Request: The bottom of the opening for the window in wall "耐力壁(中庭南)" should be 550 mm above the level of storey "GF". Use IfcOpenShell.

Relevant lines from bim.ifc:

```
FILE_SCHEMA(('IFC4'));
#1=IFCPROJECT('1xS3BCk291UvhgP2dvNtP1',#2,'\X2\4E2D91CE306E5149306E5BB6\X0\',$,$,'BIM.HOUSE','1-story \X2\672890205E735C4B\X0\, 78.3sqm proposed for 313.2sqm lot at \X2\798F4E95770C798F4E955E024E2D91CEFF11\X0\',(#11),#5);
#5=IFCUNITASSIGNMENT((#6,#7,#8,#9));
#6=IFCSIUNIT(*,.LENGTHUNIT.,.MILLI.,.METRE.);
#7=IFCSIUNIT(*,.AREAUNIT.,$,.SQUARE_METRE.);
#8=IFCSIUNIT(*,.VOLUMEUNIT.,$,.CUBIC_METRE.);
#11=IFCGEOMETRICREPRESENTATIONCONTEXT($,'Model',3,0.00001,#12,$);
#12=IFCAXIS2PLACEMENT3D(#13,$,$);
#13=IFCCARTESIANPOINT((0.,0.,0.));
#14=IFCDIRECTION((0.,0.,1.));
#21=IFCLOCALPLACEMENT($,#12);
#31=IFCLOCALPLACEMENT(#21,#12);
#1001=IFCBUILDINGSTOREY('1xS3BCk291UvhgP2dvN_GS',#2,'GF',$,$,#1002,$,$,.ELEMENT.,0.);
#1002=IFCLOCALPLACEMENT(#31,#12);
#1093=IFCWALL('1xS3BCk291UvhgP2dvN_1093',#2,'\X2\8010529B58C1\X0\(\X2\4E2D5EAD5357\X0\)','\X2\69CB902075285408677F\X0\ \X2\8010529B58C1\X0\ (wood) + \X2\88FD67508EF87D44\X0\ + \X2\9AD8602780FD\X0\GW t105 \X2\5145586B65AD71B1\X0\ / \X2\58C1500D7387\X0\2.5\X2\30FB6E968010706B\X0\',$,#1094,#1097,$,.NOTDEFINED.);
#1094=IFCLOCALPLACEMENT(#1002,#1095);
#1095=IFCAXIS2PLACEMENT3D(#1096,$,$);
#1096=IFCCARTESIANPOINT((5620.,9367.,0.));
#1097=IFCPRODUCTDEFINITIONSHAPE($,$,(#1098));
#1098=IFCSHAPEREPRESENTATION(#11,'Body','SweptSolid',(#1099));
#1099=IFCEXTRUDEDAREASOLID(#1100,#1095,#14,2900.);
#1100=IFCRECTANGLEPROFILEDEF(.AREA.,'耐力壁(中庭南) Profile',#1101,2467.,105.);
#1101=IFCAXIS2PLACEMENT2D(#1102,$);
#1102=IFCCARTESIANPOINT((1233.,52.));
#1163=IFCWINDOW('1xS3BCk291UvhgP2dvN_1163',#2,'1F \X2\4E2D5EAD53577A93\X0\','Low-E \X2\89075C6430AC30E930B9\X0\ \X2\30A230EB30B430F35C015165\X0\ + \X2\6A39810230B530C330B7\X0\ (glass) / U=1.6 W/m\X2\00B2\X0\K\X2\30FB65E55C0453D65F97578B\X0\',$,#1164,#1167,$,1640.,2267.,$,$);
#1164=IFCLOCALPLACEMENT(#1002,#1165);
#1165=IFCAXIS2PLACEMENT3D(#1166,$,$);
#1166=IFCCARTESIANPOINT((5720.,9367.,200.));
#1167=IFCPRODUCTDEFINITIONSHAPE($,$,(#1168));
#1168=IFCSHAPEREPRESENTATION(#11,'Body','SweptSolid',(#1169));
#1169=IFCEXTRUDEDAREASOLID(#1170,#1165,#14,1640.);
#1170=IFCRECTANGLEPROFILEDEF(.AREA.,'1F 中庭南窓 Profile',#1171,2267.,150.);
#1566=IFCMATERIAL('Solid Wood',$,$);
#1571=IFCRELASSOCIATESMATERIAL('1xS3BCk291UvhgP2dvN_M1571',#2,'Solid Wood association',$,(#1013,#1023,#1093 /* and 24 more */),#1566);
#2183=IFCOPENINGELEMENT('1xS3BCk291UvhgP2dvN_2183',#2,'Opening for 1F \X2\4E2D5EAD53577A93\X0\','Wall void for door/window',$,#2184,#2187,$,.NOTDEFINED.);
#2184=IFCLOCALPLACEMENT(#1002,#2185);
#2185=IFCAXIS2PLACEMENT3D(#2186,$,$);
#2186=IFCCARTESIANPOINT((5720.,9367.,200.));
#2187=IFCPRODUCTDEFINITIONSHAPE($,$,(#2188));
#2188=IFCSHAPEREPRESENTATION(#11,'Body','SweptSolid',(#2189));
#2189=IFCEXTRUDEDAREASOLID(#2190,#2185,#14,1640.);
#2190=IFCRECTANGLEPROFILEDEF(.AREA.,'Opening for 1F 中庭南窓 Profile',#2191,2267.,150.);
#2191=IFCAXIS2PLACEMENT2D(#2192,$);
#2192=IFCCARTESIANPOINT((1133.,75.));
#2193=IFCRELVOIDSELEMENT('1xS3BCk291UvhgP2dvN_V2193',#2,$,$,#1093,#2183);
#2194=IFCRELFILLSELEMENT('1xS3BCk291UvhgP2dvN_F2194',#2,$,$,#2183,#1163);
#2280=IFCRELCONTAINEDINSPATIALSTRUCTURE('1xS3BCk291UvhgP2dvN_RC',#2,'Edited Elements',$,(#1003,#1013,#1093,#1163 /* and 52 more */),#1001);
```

```python
import numpy as np
import ifcopenshell
import ifcopenshell.api.geometry
import ifcopenshell.geom
import ifcopenshell.util.element
import ifcopenshell.util.placement
import ifcopenshell.util.shape
import ifcopenshell.util.unit

model = ifcopenshell.open("bim.ifc")
unit_scale = ifcopenshell.util.unit.calculate_unit_scale(model)

window = model.by_id(1163)
opening = window.FillsVoids[0].RelatingOpeningElement
storey = ifcopenshell.util.element.get_container(window, ifc_class="IfcBuildingStorey")
level = ifcopenshell.util.placement.get_local_placement(storey.ObjectPlacement)[2, 3]

# The opening's origin need not be at the sill, so measure its lowest point.
shape = ifcopenshell.geom.create_shape(ifcopenshell.geom.settings(), opening)
bottom = ifcopenshell.util.shape.get_shape_bottom_elevation(shape, shape.geometry) / unit_scale
dz = level + 550.0 - bottom

shift = np.array([0.0, 0.0, dz])
# The window is not placed relative to its opening, so move both.
for product in (opening, window):
    matrix = ifcopenshell.util.placement.get_local_placement(product.ObjectPlacement)
    matrix[:3, 3] += shift
    ifcopenshell.api.geometry.edit_object_placement(model, product=product, matrix=matrix, is_si=False)

print(f"moved by {dz * unit_scale:+.3f} m")

model.write("bim_rev.ifc")
```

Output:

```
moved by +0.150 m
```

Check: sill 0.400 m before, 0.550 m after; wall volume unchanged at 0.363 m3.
